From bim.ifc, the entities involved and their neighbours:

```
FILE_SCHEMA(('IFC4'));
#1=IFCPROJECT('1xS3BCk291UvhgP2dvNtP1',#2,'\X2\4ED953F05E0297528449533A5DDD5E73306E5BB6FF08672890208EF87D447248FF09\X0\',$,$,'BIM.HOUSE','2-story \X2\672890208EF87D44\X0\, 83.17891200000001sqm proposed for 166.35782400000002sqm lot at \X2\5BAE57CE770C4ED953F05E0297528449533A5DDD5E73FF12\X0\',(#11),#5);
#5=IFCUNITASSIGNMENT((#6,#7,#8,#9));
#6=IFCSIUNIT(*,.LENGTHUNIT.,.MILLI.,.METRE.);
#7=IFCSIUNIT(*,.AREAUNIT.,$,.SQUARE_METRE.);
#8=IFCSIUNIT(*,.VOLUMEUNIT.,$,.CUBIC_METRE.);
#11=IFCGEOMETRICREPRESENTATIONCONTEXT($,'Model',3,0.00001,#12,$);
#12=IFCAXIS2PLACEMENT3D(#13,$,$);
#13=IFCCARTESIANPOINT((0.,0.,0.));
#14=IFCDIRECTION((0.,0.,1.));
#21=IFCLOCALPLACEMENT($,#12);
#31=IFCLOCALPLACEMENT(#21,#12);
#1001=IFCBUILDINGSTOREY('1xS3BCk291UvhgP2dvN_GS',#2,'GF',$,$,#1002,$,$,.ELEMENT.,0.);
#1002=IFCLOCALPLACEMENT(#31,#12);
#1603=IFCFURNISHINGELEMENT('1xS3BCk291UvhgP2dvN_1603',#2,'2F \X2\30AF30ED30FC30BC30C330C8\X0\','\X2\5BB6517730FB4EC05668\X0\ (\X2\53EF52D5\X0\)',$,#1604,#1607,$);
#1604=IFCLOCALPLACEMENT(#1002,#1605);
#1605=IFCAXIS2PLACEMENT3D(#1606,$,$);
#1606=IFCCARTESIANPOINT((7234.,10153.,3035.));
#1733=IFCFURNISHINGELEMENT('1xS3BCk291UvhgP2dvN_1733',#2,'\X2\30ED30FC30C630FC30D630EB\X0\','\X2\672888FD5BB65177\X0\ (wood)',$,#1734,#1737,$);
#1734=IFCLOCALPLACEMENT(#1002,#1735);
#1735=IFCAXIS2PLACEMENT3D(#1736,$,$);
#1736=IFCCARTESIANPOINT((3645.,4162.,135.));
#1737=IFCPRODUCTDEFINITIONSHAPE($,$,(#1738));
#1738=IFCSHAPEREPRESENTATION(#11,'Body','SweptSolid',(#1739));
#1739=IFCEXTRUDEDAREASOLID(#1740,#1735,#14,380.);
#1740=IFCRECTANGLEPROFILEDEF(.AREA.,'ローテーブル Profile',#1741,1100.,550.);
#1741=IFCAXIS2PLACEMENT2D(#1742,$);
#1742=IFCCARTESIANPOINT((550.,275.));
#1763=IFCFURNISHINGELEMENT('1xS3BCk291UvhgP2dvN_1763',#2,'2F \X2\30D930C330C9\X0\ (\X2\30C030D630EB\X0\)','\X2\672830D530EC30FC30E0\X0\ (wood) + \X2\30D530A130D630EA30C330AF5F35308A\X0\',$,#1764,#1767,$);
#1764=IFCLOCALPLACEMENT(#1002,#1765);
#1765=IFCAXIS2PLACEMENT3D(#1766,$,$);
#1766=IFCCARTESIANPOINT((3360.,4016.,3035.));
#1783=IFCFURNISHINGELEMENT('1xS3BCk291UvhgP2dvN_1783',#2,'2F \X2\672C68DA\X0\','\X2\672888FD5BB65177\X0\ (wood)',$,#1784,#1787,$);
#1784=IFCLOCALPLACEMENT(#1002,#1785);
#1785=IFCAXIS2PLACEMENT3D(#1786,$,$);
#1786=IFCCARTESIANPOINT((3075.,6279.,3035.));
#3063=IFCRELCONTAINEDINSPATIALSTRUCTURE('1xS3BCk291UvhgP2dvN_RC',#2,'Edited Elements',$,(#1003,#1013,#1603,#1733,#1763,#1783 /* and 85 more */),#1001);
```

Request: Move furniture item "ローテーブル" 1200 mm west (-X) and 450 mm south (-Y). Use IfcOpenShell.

```python
import ifcopenshell
import ifcopenshell.api.geometry
import ifcopenshell.util.placement
import ifcopenshell.util.unit

model = ifcopenshell.open("bim.ifc")
unit_scale = ifcopenshell.util.unit.calculate_unit_scale(model)

item = model.by_id(1733)
matrix = ifcopenshell.util.placement.get_local_placement(item.ObjectPlacement)
matrix[0, 3] -= 1.2 / unit_scale
matrix[1, 3] -= 0.45 / unit_scale
ifcopenshell.api.geometry.edit_object_placement(model, product=item, matrix=matrix, is_si=False)

print(ifcopenshell.util.placement.get_local_placement(item.ObjectPlacement).round(3) + 0.0)

model.write("bim_v2.ifc")
```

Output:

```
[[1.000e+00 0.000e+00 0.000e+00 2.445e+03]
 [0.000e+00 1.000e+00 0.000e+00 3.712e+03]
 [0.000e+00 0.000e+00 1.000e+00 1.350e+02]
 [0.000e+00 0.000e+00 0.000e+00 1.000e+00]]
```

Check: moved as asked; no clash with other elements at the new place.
